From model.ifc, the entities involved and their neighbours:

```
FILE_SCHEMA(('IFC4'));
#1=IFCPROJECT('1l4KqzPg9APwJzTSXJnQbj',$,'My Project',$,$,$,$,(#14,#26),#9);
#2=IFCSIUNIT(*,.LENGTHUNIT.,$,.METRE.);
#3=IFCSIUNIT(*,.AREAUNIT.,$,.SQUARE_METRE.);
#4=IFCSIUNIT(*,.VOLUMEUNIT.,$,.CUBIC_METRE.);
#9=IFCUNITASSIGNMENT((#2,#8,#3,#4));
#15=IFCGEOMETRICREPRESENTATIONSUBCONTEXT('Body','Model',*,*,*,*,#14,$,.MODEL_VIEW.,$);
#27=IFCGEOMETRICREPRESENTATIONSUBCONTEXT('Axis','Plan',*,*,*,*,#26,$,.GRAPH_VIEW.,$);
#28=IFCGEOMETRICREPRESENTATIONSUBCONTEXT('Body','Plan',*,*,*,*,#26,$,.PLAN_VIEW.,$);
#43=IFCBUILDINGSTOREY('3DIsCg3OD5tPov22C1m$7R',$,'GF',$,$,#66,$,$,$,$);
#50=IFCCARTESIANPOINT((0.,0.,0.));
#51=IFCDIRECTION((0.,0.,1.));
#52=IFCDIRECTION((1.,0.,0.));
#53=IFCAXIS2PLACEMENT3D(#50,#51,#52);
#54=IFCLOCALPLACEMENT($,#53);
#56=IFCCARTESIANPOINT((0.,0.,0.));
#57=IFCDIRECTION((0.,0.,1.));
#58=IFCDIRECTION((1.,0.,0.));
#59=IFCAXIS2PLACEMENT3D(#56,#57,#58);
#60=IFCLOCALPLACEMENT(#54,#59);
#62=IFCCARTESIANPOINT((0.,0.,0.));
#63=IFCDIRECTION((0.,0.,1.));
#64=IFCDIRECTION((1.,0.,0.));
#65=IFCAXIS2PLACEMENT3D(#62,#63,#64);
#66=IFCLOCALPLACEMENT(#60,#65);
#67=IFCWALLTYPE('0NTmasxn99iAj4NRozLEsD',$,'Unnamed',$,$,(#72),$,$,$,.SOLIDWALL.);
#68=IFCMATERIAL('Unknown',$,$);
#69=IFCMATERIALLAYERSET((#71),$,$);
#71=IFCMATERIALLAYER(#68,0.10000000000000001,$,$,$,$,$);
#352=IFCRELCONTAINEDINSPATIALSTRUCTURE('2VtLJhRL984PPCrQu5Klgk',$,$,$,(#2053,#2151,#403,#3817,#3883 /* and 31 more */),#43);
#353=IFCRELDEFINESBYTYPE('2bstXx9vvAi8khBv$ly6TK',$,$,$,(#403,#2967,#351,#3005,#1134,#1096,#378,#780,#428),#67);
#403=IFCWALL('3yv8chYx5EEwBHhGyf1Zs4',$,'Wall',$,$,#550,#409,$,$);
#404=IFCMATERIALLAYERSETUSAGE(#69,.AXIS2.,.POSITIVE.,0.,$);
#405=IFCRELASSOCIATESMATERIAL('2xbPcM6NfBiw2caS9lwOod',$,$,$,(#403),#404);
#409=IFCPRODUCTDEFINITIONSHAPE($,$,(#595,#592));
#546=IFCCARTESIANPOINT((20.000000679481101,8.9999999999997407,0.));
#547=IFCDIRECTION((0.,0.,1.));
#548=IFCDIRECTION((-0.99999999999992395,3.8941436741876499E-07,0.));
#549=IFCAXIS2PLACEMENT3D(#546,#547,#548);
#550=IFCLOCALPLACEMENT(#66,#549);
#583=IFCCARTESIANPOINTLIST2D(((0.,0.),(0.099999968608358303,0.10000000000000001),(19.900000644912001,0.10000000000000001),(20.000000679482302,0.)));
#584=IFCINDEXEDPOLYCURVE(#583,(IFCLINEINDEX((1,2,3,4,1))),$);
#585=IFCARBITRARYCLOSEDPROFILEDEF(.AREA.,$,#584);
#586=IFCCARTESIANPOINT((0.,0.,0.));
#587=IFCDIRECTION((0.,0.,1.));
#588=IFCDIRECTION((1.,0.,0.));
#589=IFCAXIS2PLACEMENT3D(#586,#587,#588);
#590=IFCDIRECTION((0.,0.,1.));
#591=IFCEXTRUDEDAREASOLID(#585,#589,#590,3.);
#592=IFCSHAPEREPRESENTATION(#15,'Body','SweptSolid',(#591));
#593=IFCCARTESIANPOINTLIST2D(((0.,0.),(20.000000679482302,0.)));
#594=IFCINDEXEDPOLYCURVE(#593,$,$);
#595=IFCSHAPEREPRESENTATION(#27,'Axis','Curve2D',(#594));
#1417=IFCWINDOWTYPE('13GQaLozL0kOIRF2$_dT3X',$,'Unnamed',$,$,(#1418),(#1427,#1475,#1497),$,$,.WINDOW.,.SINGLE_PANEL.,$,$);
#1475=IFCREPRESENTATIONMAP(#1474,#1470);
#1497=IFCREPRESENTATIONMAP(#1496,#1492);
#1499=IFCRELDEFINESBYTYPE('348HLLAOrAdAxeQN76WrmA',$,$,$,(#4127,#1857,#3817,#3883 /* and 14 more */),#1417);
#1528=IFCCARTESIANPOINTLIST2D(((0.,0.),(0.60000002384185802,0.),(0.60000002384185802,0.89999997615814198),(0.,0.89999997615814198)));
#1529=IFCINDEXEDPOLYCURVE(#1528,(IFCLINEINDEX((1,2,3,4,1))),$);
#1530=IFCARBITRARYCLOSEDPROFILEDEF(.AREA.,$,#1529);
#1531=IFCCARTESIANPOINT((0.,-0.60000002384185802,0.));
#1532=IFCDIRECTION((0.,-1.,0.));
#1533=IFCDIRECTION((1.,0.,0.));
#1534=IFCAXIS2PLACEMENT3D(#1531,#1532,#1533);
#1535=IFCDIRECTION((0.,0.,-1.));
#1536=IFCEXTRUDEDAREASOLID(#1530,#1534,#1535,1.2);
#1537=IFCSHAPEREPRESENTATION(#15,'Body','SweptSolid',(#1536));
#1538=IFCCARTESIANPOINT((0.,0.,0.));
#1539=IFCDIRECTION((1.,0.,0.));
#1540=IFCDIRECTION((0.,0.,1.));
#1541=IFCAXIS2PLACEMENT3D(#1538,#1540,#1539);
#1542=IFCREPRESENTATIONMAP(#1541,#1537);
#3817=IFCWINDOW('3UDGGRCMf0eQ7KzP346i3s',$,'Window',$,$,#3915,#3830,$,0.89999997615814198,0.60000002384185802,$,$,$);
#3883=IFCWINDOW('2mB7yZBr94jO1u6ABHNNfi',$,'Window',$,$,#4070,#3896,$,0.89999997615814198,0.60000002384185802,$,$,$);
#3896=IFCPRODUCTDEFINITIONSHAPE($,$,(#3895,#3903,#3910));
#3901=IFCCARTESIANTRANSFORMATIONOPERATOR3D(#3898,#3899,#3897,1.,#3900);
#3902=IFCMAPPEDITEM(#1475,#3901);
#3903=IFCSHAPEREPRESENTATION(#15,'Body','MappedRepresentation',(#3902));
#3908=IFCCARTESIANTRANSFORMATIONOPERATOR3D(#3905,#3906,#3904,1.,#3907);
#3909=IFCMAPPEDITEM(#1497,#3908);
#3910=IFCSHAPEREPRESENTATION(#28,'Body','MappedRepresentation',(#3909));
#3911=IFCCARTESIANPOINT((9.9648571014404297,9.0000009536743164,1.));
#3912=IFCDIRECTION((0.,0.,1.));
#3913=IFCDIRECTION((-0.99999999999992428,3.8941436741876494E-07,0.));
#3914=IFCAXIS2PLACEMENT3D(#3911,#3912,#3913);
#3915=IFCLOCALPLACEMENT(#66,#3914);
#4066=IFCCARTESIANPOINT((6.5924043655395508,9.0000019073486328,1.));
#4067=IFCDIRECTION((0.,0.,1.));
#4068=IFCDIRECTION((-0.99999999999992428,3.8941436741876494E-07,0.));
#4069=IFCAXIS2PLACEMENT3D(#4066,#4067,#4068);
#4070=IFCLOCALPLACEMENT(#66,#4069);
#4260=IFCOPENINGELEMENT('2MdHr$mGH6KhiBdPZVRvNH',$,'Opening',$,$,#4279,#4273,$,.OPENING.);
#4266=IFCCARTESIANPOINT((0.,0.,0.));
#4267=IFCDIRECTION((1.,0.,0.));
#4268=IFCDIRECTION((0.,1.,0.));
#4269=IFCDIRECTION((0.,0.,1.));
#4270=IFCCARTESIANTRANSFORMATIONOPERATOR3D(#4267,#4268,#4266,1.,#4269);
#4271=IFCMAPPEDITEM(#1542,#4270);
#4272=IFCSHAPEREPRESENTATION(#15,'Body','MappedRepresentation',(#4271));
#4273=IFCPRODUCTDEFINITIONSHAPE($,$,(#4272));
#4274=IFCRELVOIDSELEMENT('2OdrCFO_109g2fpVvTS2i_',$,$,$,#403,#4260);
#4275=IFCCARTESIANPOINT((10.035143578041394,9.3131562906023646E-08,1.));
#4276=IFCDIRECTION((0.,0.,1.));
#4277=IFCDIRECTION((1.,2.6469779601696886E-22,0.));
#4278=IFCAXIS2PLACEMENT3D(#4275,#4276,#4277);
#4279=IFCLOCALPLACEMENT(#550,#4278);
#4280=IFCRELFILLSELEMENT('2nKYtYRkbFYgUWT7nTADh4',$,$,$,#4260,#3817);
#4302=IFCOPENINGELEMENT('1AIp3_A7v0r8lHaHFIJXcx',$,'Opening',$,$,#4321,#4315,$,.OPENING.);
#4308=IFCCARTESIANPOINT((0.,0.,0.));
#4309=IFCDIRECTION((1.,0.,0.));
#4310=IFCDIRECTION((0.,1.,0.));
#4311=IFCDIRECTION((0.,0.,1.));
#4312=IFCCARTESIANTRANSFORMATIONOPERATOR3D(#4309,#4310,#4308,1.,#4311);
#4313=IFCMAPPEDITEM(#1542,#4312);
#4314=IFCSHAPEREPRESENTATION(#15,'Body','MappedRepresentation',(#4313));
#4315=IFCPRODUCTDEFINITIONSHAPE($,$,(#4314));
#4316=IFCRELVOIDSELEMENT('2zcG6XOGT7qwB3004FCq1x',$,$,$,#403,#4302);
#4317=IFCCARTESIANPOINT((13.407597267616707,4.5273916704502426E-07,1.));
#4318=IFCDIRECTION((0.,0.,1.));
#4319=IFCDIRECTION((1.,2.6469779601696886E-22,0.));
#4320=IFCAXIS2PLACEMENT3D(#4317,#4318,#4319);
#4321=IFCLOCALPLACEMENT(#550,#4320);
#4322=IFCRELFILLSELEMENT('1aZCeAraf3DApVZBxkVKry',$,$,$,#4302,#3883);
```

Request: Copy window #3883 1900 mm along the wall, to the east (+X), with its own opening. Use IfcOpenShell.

```python
import ifcopenshell
import ifcopenshell.api.feature
import ifcopenshell.api.geometry
import ifcopenshell.api.root
import ifcopenshell.geom
import ifcopenshell.util.element
import ifcopenshell.util.placement
import ifcopenshell.util.shape
import ifcopenshell.util.unit

model = ifcopenshell.open("model.ifc")
unit_scale = ifcopenshell.util.unit.calculate_unit_scale(model)
settings = ifcopenshell.geom.settings()


def volume(element):
    """Net volume in cubic metres, openings subtracted."""
    shape = ifcopenshell.geom.create_shape(settings, element)
    return ifcopenshell.util.shape.get_volume(shape.geometry)


window = model.by_guid("2mB7yZBr94jO1u6ABHNNfi")
opening = window.FillsVoids[0].RelatingOpeningElement
wall = opening.VoidsElements[0].RelatingBuildingElement
before = volume(wall)
shift = ifcopenshell.util.placement.get_local_placement(wall.ObjectPlacement)[:3, 0] * -1.9 / unit_scale

# copy_class copies the void relationship, type, container and properties, but no geometry.
new_opening = ifcopenshell.api.root.copy_class(model, product=opening)
new_opening.Representation = ifcopenshell.util.element.copy_deep(
    model, opening.Representation, exclude=["IfcGeometricRepresentationContext", "IfcRepresentationMap"]
)
new_window = ifcopenshell.api.root.copy_class(model, product=window)
new_window.Representation = ifcopenshell.util.element.copy_deep(
    model, window.Representation, exclude=["IfcGeometricRepresentationContext", "IfcRepresentationMap"]
)
ifcopenshell.api.feature.add_filling(model, opening=new_opening, element=new_window)

for old, new in ((opening, new_opening), (window, new_window)):
    matrix = ifcopenshell.util.placement.get_local_placement(old.ObjectPlacement)
    matrix[:3, 3] += shift
    ifcopenshell.api.geometry.edit_object_placement(model, product=new, matrix=matrix, is_si=False)

after = volume(wall)

print(f"wall volume {before:.3f} -> {after:.3f} m3")

model.write("model_edited.ifc")
```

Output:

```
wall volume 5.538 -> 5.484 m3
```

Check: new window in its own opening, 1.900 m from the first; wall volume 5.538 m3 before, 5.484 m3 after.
